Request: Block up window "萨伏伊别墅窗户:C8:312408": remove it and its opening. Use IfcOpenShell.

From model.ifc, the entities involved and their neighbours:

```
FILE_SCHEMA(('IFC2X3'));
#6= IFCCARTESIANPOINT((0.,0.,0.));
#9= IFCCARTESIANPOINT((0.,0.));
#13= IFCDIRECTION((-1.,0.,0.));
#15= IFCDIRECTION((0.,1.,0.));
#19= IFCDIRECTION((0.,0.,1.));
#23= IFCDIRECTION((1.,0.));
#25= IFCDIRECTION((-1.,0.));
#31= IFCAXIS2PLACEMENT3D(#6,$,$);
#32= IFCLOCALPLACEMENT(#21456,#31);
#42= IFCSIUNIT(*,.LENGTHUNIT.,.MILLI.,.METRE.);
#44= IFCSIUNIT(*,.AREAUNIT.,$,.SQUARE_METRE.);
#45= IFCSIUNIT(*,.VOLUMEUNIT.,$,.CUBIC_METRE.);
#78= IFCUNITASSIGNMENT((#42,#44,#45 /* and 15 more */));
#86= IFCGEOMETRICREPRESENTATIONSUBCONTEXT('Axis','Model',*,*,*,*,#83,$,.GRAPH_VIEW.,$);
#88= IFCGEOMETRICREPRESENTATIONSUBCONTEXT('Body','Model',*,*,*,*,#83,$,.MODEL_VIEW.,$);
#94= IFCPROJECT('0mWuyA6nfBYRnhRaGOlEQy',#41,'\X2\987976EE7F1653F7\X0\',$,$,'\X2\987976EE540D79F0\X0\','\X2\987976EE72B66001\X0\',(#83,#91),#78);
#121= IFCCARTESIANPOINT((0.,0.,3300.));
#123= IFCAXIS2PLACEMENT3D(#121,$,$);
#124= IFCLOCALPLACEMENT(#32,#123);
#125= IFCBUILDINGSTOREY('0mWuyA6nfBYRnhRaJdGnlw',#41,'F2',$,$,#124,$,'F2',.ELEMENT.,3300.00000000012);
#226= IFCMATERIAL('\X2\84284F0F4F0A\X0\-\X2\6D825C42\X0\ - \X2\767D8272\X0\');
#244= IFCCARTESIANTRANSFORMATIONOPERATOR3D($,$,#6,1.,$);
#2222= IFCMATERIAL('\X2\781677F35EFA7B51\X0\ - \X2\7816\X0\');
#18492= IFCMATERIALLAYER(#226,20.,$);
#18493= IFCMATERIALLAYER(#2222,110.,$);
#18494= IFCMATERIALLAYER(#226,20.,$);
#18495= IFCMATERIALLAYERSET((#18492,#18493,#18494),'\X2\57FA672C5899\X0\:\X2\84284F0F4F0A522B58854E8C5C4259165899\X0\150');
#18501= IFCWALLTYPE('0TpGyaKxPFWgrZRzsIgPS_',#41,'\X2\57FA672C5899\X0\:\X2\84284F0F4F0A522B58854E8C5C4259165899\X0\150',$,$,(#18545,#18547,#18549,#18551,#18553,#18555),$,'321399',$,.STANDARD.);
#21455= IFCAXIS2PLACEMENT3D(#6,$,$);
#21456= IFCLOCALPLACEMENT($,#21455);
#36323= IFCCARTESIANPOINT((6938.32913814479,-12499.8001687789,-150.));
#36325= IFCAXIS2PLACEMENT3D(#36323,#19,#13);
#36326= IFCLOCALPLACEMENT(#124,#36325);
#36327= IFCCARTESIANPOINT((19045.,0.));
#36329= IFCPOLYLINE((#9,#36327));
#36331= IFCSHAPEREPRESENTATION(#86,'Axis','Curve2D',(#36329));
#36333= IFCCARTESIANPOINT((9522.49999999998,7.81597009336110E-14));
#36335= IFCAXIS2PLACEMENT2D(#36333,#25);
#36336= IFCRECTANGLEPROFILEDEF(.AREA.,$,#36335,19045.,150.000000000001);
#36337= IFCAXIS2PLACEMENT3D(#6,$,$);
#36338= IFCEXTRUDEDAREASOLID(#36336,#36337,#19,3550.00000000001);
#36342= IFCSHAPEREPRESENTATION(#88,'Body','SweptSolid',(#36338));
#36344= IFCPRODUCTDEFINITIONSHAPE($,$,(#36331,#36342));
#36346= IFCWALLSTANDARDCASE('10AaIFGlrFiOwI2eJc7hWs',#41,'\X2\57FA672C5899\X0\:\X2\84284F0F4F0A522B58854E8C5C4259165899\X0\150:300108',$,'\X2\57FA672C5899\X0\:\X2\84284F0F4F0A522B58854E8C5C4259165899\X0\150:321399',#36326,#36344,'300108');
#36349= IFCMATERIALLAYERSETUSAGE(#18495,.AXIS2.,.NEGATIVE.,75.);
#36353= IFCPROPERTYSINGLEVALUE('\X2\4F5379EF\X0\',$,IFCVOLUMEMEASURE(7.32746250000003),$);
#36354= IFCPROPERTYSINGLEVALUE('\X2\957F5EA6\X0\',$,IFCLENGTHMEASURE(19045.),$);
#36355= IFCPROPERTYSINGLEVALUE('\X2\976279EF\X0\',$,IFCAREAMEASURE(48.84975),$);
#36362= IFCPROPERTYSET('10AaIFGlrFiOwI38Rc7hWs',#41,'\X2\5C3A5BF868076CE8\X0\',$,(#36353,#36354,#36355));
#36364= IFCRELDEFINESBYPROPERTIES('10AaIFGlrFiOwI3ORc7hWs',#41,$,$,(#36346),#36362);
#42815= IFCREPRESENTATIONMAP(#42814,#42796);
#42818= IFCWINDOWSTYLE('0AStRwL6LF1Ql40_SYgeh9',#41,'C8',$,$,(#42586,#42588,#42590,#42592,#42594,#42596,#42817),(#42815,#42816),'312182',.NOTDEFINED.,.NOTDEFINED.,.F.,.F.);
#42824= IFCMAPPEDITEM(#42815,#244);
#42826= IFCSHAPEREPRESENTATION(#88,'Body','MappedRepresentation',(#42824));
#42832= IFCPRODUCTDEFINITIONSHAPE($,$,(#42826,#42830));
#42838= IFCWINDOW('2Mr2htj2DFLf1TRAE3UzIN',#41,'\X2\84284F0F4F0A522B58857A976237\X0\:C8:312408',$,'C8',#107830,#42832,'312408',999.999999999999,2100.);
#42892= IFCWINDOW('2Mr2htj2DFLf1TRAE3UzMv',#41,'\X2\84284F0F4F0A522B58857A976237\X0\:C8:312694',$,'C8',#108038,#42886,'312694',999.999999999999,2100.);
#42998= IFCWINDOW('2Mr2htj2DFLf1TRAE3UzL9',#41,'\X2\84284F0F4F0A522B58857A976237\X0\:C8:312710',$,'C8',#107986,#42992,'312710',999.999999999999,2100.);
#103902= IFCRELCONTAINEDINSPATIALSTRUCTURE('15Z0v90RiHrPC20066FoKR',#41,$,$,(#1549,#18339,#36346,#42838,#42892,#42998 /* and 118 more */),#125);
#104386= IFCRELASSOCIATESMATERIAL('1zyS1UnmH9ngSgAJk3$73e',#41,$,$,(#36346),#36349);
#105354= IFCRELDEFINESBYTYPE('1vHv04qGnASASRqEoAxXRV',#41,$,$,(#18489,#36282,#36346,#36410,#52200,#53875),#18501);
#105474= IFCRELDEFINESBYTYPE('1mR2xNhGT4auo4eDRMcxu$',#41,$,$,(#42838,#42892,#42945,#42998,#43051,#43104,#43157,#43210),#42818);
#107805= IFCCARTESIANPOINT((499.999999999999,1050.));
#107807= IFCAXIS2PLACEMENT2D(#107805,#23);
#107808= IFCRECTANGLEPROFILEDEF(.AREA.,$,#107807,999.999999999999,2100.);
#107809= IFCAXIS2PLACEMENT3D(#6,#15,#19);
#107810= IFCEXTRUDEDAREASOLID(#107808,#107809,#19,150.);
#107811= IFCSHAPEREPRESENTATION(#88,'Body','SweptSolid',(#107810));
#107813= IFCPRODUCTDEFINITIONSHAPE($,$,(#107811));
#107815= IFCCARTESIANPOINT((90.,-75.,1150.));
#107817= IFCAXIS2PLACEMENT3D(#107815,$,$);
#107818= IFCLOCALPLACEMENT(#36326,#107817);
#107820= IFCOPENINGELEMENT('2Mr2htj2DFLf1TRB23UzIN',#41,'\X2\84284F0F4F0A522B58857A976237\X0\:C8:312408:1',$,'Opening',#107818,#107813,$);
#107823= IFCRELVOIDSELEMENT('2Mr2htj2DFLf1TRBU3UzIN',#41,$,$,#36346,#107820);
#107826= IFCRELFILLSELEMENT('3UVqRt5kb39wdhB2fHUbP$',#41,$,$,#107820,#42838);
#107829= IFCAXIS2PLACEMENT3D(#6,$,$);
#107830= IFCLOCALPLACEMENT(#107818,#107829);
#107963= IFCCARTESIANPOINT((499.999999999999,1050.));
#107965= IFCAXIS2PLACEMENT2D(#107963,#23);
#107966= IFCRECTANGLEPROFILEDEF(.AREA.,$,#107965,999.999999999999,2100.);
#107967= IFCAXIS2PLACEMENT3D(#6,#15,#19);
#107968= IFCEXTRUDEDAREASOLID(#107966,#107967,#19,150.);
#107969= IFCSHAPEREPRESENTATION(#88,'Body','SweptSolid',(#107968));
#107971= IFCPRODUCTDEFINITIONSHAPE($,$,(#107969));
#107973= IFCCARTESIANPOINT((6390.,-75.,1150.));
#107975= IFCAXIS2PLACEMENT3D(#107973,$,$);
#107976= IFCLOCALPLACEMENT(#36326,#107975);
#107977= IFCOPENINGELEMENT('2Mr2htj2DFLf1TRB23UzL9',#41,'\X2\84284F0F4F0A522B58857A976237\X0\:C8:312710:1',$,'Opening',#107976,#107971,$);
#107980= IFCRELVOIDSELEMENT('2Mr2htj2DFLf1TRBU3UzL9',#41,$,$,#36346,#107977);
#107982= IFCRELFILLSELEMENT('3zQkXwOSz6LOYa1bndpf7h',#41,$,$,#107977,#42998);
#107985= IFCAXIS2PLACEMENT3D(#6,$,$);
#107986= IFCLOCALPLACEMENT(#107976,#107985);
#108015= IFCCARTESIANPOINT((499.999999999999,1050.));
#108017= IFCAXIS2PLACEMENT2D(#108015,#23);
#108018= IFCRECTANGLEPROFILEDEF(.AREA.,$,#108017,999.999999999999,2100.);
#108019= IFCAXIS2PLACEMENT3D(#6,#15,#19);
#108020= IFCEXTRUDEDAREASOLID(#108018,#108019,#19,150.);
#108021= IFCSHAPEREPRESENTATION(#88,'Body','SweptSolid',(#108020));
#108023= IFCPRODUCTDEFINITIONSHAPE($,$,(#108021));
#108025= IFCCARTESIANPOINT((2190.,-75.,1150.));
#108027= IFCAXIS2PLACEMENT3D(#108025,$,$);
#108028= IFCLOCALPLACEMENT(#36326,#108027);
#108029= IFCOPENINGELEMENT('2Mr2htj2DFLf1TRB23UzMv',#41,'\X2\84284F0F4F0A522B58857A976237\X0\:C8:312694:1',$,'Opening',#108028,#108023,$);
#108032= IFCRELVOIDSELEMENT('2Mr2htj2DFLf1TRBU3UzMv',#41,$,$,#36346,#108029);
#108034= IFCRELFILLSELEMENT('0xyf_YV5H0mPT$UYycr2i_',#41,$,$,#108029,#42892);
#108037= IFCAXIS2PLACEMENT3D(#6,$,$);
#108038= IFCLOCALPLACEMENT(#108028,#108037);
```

```python
import ifcopenshell
import ifcopenshell.api.feature
import ifcopenshell.api.pset
import ifcopenshell.api.root
import ifcopenshell.geom
import ifcopenshell.util.element
import ifcopenshell.util.shape
import ifcopenshell.util.unit

model = ifcopenshell.open("model.ifc")
area_scale = ifcopenshell.util.unit.calculate_unit_scale(model, "AREAUNIT")
volume_scale = ifcopenshell.util.unit.calculate_unit_scale(model, "VOLUMEUNIT")
settings = ifcopenshell.geom.settings()


def volume(element):
    """Net volume in cubic metres, openings subtracted."""
    shape = ifcopenshell.geom.create_shape(settings, element)
    return ifcopenshell.util.shape.get_volume(shape.geometry)


window = model.by_guid("2Mr2htj2DFLf1TRAE3UzIN")
opening = window.FillsVoids[0].RelatingOpeningElement
wall = opening.VoidsElements[0].RelatingBuildingElement
before = volume(wall)

ifcopenshell.api.root.remove_product(model, product=window)
ifcopenshell.api.feature.remove_feature(model, feature=opening)

after = volume(wall)
thickness = 0.15  # wall thickness in metres

# Update the wall's stored quantities.
pset = model.by_id(ifcopenshell.util.element.get_pset(wall, "尺寸标注", should_inherit=False)["id"])
ifcopenshell.api.pset.edit_pset(model, pset=pset, properties={
    "体积": model.create_entity("IfcVolumeMeasure", after / volume_scale),
    "面积": model.create_entity("IfcAreaMeasure", after / thickness / area_scale),
})

print(f"wall volume {before:.3f} -> {after:.3f} m3")

model.write("model_edited.ifc")
```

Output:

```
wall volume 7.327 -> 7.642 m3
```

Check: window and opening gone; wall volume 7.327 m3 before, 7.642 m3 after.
